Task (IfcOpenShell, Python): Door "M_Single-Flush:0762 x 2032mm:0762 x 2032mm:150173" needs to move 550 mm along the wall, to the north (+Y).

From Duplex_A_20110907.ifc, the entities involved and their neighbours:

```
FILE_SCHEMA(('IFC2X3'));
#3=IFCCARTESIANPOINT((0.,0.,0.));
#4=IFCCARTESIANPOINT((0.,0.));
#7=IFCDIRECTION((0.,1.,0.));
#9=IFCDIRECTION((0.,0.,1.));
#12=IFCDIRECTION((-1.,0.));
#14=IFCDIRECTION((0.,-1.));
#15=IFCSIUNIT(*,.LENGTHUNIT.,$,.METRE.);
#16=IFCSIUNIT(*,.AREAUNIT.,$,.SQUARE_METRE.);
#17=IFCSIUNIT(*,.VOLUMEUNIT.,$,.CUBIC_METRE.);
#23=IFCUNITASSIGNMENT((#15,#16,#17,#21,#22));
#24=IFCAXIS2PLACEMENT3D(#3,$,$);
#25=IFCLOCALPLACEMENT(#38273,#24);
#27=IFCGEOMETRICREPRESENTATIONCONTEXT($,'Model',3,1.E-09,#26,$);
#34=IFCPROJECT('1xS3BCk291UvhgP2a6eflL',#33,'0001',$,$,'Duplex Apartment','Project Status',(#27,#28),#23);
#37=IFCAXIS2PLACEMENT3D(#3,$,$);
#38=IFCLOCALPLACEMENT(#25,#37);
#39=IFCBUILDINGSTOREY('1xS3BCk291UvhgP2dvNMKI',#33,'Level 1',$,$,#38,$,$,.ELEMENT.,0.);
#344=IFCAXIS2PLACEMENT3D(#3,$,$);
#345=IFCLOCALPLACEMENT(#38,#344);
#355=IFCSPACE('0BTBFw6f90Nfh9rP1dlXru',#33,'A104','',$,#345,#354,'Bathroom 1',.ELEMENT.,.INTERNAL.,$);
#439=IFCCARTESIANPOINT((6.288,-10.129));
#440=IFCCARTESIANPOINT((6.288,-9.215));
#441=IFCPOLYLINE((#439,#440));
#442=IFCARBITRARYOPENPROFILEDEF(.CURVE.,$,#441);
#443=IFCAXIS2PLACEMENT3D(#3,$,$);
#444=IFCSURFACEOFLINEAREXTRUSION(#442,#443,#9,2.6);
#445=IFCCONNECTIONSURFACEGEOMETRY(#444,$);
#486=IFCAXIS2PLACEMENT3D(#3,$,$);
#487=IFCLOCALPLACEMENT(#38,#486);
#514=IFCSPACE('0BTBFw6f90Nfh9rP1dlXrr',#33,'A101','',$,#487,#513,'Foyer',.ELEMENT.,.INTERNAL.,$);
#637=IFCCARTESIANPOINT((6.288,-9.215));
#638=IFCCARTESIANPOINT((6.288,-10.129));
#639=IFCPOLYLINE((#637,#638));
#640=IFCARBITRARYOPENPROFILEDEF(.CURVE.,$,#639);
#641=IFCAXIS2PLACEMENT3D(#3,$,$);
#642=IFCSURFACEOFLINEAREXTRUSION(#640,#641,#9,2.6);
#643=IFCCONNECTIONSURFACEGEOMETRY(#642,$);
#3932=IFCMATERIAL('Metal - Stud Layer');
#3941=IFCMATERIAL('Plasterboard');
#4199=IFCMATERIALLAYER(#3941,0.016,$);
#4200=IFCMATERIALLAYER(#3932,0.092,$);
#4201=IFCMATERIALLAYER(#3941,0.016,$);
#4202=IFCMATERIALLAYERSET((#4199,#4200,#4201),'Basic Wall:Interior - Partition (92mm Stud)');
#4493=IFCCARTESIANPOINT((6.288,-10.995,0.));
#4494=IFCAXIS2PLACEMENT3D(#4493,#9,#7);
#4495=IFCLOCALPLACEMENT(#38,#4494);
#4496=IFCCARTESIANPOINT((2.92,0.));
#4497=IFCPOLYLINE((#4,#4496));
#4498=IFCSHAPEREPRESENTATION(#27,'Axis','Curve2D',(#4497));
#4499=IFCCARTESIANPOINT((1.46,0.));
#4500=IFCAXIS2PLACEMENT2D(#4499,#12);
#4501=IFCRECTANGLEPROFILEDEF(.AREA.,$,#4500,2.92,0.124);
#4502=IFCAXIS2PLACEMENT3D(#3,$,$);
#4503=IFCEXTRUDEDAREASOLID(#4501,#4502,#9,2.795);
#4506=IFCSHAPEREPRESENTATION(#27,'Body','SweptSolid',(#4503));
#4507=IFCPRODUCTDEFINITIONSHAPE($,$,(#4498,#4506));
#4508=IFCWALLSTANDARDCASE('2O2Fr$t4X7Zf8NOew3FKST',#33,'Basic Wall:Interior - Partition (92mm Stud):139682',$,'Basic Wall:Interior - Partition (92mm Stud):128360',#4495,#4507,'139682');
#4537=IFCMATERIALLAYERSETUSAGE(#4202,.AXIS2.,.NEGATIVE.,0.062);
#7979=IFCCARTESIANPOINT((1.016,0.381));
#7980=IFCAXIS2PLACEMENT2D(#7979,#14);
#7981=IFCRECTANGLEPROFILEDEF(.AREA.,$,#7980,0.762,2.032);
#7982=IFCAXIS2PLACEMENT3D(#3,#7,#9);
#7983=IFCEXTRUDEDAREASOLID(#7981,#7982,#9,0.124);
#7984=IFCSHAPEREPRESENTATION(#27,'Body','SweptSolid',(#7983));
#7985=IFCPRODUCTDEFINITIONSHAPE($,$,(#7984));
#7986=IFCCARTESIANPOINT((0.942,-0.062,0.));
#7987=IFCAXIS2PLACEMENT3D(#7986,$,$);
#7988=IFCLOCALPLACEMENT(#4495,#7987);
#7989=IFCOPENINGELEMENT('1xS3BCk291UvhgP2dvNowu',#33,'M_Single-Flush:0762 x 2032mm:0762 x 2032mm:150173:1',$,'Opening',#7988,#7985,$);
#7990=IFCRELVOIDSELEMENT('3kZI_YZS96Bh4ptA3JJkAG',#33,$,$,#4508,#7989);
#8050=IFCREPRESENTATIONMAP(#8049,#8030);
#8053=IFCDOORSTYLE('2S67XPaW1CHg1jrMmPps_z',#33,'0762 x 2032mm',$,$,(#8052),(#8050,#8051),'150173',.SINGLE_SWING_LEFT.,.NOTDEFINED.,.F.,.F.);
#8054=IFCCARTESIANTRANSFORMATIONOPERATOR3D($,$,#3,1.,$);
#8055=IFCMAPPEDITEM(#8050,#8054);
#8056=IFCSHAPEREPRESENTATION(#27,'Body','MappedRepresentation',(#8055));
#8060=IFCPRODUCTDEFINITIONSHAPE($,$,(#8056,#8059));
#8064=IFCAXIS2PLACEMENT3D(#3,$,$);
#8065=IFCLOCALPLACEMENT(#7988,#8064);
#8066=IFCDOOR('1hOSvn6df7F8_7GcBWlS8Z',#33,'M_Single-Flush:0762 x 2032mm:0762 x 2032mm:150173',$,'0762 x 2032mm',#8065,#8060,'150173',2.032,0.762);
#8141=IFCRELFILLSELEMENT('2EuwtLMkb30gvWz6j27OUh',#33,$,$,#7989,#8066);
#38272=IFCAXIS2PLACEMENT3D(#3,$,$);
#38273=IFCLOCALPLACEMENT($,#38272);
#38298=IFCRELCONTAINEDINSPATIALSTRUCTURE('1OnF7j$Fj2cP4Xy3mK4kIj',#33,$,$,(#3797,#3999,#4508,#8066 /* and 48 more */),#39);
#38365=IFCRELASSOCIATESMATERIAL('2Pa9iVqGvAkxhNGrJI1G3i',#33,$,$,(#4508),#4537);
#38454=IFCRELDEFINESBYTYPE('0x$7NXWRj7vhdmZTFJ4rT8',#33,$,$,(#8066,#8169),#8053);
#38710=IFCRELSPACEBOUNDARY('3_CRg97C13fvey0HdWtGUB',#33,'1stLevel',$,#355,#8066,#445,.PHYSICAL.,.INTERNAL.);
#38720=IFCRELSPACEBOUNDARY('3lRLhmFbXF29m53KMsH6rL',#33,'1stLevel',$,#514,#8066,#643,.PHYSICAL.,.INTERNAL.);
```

```python
import numpy as np
import ifcopenshell
import ifcopenshell.api.geometry
import ifcopenshell.util.placement

model = ifcopenshell.open("Duplex_A_20110907.ifc")

door = model.by_guid("1hOSvn6df7F8_7GcBWlS8Z")
opening = door.FillsVoids[0].RelatingOpeningElement
wall = opening.VoidsElements[0].RelatingBuildingElement

wall_matrix = ifcopenshell.util.placement.get_local_placement(wall.ObjectPlacement)
shift = wall_matrix[:3, 0] * 0.55
before = ifcopenshell.util.placement.get_local_placement(door.ObjectPlacement)[:3, 3].copy()

# The door is placed relative to its opening, so it follows when the opening moves.
matrix = ifcopenshell.util.placement.get_local_placement(opening.ObjectPlacement)
matrix[:3, 3] += shift
ifcopenshell.api.geometry.edit_object_placement(
    model, product=opening, matrix=matrix, is_si=False, should_transform_children=True
)

# Space boundary surfaces are stored in each space's coordinates; move them too.
for rel in door.ProvidesBoundaries:
    if not rel.ConnectionGeometry:
        continue
    surface = rel.ConnectionGeometry.SurfaceOnRelatingElement
    space_matrix = ifcopenshell.util.placement.get_local_placement(rel.RelatingSpace.ObjectPlacement)
    point = np.array(surface.Position.Location.Coordinates) + space_matrix[:3, :3].T @ shift
    surface.Position = model.createIfcAxis2Placement3D(
        model.createIfcCartesianPoint(point.tolist()), surface.Position.Axis, surface.Position.RefDirection
    )

after = ifcopenshell.util.placement.get_local_placement(door.ObjectPlacement)[:3, 3]
print("door moved by", (after - before).round(3) + 0.0)

model.write("Duplex_A_20110907_rev.ifc")
```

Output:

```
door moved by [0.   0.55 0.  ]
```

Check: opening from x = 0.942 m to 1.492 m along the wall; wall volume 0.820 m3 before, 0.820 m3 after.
